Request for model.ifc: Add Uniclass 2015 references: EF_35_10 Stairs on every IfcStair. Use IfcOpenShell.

First a look at what the model holds.

```python
import ifcopenshell

model = ifcopenshell.open("model.ifc")
print(model.schema)
print("classifications:", [c.Name for c in model.by_type("IfcClassification")])
for ifc_class in ("IfcDoor", "IfcRoof", "IfcStair", "IfcWall", "IfcWindow"):
    print(ifc_class, len(model.by_type(ifc_class)))
```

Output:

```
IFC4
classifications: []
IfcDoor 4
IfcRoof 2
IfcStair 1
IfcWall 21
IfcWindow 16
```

```python
import ifcopenshell
import ifcopenshell.api.classification

model = ifcopenshell.open("model.ifc")

system = ifcopenshell.api.classification.add_classification(model, classification="Uniclass 2015")

codes = {
    "IfcStair": ("EF_35_10", "Stairs"),
}
for ifc_class, (code, name) in codes.items():
    products = model.by_type(ifc_class)
    ifcopenshell.api.classification.add_reference(
        model, products=products, classification=system, identification=code, name=name
    )
    print(code, len(products))

model.write("model_rev.ifc")
```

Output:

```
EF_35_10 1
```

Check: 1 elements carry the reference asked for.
